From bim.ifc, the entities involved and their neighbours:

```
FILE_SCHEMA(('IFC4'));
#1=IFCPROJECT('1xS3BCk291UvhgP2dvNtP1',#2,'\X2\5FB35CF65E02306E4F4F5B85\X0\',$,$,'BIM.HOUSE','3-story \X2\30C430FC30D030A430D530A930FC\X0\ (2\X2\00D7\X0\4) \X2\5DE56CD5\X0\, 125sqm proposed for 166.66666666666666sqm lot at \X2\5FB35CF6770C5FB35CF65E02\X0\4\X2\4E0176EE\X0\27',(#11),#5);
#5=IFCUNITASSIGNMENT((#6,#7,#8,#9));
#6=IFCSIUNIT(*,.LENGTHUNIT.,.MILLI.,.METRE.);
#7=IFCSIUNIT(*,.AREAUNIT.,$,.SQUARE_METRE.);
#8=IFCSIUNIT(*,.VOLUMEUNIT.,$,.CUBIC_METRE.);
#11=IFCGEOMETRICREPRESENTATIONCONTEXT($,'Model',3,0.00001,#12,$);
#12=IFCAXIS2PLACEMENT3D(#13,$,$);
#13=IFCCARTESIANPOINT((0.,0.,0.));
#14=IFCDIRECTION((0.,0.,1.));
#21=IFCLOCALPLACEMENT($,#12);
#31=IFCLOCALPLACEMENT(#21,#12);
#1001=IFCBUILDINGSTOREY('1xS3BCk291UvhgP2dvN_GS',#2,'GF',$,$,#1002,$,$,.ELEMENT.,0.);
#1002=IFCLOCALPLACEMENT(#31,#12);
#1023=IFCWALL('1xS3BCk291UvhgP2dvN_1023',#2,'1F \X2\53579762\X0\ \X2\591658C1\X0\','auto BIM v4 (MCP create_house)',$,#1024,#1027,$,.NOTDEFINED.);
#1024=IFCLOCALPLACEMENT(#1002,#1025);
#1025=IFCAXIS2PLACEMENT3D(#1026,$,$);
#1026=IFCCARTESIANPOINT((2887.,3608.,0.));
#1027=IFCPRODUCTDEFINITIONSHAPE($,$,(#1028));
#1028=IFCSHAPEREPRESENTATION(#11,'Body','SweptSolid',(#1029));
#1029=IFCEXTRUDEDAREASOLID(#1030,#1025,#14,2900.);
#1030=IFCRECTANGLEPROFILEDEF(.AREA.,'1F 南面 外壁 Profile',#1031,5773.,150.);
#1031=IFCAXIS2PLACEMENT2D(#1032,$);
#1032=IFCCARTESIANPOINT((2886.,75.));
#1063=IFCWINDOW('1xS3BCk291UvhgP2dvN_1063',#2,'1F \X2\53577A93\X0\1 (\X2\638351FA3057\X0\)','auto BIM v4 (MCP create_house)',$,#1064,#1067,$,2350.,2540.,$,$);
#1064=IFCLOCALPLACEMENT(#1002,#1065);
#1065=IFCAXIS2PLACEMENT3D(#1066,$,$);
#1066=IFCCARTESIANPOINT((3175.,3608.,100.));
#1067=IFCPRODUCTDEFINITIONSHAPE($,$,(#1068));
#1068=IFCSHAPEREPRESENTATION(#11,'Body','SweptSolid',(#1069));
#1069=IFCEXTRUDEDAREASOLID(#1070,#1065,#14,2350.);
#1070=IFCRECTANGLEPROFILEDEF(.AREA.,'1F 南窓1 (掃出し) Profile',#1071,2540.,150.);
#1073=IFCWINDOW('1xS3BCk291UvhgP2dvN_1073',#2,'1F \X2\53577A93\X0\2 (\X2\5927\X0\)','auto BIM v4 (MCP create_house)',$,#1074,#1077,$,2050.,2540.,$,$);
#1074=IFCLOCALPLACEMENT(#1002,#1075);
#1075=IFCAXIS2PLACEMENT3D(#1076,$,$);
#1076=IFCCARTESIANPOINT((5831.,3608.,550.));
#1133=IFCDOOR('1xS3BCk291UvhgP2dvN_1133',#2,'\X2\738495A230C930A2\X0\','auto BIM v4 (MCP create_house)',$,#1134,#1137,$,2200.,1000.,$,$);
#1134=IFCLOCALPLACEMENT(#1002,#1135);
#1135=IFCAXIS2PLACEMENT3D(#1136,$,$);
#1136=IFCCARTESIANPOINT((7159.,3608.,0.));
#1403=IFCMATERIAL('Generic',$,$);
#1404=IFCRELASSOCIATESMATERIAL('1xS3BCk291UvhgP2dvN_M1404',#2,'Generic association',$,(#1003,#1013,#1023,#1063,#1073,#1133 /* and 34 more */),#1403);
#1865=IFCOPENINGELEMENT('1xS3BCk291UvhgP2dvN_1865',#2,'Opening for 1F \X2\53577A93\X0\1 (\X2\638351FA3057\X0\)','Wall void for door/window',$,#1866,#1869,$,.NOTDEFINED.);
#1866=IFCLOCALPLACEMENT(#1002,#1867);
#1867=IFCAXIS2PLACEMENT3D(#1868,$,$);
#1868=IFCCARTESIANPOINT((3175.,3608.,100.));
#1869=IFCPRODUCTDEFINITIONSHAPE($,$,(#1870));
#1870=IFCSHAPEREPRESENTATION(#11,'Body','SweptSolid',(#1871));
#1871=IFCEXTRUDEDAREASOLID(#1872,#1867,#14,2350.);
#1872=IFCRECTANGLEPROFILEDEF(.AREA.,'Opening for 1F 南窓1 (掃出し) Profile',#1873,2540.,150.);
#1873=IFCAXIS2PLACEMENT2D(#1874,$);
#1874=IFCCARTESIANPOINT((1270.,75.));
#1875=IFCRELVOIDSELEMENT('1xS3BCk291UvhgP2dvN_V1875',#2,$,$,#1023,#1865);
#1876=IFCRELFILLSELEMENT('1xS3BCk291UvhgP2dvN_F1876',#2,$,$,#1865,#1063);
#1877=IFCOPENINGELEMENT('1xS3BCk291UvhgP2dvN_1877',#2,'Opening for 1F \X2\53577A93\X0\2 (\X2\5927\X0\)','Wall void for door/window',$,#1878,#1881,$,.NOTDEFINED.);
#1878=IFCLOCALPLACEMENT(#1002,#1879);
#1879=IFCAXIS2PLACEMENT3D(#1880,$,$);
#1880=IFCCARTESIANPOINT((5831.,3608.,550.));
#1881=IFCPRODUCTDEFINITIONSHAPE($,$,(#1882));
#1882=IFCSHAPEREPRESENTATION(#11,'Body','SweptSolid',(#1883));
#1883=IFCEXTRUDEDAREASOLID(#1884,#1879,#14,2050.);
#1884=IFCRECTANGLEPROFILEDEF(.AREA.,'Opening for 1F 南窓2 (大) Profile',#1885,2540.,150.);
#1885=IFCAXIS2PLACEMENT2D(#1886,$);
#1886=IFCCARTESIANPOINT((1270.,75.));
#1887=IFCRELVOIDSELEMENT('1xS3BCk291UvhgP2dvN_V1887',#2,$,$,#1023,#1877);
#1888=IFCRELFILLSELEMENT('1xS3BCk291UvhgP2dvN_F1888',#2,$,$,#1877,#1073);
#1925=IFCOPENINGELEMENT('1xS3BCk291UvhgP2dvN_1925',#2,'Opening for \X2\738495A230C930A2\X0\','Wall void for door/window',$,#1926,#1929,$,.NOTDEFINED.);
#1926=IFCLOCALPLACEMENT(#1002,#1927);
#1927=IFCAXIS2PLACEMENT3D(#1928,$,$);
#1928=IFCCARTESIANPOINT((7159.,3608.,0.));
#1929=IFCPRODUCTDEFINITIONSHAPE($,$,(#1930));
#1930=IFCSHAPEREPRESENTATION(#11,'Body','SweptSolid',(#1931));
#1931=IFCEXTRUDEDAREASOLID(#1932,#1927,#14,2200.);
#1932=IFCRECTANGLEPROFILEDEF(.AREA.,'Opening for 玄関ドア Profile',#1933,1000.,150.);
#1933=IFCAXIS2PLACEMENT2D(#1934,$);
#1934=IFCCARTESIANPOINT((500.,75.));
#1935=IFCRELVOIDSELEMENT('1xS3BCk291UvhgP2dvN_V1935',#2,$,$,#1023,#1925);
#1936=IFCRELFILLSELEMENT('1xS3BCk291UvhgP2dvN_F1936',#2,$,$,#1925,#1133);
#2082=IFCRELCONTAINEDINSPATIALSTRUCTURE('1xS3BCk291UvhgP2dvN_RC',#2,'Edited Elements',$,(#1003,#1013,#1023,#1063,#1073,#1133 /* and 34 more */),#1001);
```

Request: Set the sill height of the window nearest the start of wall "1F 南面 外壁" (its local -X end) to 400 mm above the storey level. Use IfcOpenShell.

```python
import numpy as np
import ifcopenshell
import ifcopenshell.api.geometry
import ifcopenshell.geom
import ifcopenshell.util.element
import ifcopenshell.util.placement
import ifcopenshell.util.shape
import ifcopenshell.util.unit

model = ifcopenshell.open("bim.ifc")
unit_scale = ifcopenshell.util.unit.calculate_unit_scale(model)

window = model.by_guid("1xS3BCk291UvhgP2dvN_1063")
opening = window.FillsVoids[0].RelatingOpeningElement
storey = ifcopenshell.util.element.get_container(window, ifc_class="IfcBuildingStorey")
level = ifcopenshell.util.placement.get_local_placement(storey.ObjectPlacement)[2, 3]

# The opening's origin need not be at the sill, so measure its lowest point.
shape = ifcopenshell.geom.create_shape(ifcopenshell.geom.settings(), opening)
bottom = ifcopenshell.util.shape.get_shape_bottom_elevation(shape, shape.geometry) / unit_scale
dz = level + 0.4 / unit_scale - bottom

shift = np.array([0.0, 0.0, dz])
# The window is not placed relative to its opening, so move both.
for product in (opening, window):
    matrix = ifcopenshell.util.placement.get_local_placement(product.ObjectPlacement)
    matrix[:3, 3] += shift
    ifcopenshell.api.geometry.edit_object_placement(model, product=product, matrix=matrix, is_si=False)

print(f"moved by {dz * unit_scale:+.3f} m")

model.write("bim_edited.ifc")
```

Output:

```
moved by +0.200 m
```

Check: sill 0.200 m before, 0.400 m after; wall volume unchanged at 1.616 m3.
